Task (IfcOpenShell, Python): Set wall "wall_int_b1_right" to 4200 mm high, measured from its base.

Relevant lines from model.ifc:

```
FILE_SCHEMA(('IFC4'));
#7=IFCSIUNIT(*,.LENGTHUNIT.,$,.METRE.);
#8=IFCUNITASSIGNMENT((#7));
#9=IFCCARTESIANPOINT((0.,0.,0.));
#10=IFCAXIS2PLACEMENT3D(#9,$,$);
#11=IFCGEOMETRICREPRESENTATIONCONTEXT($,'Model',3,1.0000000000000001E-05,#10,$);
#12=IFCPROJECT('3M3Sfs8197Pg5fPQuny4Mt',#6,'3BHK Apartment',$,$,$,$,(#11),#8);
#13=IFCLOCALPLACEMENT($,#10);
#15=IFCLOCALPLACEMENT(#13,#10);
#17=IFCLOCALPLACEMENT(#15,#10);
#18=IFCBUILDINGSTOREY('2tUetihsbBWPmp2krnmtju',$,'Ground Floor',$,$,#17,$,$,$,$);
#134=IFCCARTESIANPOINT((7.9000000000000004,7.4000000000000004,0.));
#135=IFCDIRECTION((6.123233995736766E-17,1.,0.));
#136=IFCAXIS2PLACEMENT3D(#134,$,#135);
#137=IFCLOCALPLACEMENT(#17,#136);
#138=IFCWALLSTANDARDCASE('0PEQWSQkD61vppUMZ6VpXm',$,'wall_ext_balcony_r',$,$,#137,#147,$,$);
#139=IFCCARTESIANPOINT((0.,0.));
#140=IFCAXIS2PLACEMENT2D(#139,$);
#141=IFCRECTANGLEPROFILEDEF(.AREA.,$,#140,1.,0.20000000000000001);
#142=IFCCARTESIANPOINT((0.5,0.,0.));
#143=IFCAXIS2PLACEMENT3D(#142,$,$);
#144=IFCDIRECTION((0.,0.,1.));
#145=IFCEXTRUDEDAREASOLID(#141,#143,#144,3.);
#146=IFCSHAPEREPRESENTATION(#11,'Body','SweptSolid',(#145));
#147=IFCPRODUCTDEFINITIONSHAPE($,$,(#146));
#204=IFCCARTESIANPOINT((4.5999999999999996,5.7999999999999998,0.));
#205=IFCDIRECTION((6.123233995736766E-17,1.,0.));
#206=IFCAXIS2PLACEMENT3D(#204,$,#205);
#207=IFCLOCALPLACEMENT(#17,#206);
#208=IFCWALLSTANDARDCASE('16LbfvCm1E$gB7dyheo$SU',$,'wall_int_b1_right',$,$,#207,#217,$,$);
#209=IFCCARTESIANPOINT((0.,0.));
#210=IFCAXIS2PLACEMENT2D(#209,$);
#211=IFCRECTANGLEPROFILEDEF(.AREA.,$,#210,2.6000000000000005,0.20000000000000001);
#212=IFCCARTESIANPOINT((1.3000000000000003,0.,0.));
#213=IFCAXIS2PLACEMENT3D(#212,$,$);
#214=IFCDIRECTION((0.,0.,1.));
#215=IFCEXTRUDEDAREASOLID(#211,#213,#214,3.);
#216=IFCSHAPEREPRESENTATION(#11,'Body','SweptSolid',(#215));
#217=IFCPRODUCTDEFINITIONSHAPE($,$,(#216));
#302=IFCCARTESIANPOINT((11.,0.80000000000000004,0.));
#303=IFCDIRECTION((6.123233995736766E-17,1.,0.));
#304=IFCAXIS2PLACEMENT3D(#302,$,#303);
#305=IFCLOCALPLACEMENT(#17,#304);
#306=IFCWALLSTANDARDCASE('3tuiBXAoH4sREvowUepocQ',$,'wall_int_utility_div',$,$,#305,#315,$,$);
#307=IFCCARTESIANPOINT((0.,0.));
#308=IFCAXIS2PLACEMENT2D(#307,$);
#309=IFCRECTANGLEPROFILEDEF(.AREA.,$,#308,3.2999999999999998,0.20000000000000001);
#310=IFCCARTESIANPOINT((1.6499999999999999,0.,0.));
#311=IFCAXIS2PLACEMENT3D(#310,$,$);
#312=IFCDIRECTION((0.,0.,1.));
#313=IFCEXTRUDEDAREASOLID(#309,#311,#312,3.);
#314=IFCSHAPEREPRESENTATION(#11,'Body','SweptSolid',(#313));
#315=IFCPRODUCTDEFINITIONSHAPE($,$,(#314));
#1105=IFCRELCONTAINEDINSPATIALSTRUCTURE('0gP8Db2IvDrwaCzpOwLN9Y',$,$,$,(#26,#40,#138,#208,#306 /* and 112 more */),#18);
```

```python
import ifcopenshell
import ifcopenshell.geom
import ifcopenshell.util.shape
import ifcopenshell.util.unit

model = ifcopenshell.open("model.ifc")
unit_scale = ifcopenshell.util.unit.calculate_unit_scale(model)
settings = ifcopenshell.geom.settings()


def volume(element):
    """Net volume in cubic metres, openings subtracted."""
    shape = ifcopenshell.geom.create_shape(settings, element)
    return ifcopenshell.util.shape.get_volume(shape.geometry)


wall = model.by_guid("16LbfvCm1E$gB7dyheo$SU")
before = volume(wall)

body = next(r for r in wall.Representation.Representations if r.RepresentationIdentifier == "Body")
solid = body.Items[0]
old_height = solid.Depth
solid.Depth = 4.2 / unit_scale
after = volume(wall)

print(f"height {old_height:g} -> {solid.Depth:g}, volume {before:.3f} -> {after:.3f} m3")

model.write("model-out.ifc")
```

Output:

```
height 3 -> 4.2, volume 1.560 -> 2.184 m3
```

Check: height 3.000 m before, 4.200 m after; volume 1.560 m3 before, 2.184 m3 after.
